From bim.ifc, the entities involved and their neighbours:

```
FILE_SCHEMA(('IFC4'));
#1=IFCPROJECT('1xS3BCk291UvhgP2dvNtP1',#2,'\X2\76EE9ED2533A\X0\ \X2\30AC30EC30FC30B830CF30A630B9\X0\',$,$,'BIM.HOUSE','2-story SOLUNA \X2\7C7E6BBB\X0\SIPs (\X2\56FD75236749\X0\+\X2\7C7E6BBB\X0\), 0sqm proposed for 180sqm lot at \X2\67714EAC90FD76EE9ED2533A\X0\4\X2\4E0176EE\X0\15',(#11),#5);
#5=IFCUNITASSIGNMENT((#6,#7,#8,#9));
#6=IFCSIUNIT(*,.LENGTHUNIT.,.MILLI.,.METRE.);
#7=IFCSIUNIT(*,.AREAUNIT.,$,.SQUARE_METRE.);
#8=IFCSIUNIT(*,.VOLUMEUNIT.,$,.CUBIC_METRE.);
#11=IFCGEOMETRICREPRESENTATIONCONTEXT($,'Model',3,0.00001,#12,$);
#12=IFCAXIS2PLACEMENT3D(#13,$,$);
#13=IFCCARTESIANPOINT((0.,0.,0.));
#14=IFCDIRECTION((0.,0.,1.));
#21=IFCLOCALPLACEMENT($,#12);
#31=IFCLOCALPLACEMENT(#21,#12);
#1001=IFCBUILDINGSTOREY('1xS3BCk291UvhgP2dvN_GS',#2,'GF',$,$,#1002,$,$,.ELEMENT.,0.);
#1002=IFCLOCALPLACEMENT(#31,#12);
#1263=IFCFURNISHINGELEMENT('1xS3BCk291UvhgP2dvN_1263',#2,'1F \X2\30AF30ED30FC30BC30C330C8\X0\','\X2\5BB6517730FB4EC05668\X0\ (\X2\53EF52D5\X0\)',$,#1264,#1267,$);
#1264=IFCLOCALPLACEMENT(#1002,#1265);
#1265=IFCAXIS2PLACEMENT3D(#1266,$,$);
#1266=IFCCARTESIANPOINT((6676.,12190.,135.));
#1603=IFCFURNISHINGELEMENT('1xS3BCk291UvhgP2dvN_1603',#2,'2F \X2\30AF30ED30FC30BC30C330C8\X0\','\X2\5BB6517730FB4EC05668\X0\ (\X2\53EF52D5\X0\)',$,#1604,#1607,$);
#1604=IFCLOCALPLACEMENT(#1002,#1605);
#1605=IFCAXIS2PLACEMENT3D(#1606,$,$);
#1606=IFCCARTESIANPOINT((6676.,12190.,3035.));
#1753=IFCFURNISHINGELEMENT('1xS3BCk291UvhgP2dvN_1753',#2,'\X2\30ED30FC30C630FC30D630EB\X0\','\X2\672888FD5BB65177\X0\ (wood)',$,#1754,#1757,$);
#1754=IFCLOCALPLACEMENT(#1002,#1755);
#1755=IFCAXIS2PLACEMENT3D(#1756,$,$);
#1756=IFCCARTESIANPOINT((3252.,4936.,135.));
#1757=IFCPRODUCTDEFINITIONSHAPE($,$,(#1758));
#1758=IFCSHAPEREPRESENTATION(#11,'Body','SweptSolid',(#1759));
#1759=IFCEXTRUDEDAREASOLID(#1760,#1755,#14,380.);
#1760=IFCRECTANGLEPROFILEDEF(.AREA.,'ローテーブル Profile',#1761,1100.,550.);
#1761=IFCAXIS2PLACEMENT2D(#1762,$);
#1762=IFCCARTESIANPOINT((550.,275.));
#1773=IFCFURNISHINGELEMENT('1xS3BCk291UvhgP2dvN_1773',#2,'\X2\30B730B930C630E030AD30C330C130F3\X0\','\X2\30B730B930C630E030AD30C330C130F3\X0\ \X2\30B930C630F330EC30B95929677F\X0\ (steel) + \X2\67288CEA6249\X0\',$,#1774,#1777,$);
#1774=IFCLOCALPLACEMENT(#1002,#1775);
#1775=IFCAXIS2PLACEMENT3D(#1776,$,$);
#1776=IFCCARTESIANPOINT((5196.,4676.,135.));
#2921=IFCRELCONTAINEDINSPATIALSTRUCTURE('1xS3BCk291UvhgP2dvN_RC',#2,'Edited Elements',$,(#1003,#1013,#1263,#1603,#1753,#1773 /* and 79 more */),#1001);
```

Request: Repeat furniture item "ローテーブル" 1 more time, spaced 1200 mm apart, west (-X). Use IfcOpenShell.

```python
import numpy as np
import ifcopenshell
import ifcopenshell.api.geometry
import ifcopenshell.api.root
import ifcopenshell.util.element
import ifcopenshell.util.placement
import ifcopenshell.util.unit

model = ifcopenshell.open("bim.ifc")
unit_scale = ifcopenshell.util.unit.calculate_unit_scale(model)


def reuse_history(source, copy):
    """copy_class also copies each property set's owner history, people and application; keep the originals."""
    for rel in copy.IsDefinedBy:
        if rel.is_a("IfcRelDefinesByProperties") and (history := rel.RelatingPropertyDefinition.OwnerHistory):
            rel.RelatingPropertyDefinition.OwnerHistory = source.OwnerHistory
            ifcopenshell.util.element.remove_deep2(model, history)


source = model.by_guid("1xS3BCk291UvhgP2dvN_1753")
base = ifcopenshell.util.placement.get_local_placement(source.ObjectPlacement)
step = np.array([-1.0, 0.0, 0.0]) * 1.2 / unit_scale

for i in range(1, 2):
    copy = ifcopenshell.api.root.copy_class(model, product=source)
    copy.Representation = ifcopenshell.util.element.copy_deep(
        model, source.Representation, exclude=["IfcGeometricRepresentationContext", "IfcRepresentationMap"]
    )
    reuse_history(source, copy)
    matrix = base.copy()
    matrix[:3, 3] += i * step
    print("added at", matrix[:3, 3].round(3) + 0.0)
    ifcopenshell.api.geometry.edit_object_placement(model, product=copy, matrix=matrix, is_si=False)

model.write("bim_rev.ifc")
```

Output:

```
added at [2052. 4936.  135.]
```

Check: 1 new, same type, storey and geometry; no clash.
